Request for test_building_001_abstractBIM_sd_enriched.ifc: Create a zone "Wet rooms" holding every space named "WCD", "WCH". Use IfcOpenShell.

First a look at what the model holds.

```python
import ifcopenshell

model = ifcopenshell.open("test_building_001_abstractBIM_sd_enriched.ifc")
print(model.schema)
seen = {}
for space in model.by_type("IfcSpace"):
    seen[space.LongName] = seen.get(space.LongName, 0) + 1
for name, count in sorted(seen.items(), key=str):
    print(count, "x", name)
print("zones:", [z.Name for z in model.by_type("IfcZone")][:20])
```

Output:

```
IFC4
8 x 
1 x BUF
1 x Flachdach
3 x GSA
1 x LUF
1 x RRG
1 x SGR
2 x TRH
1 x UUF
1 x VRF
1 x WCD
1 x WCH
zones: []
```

```python
import ifcopenshell
import ifcopenshell.api.group
import ifcopenshell.api.root

model = ifcopenshell.open("test_building_001_abstractBIM_sd_enriched.ifc")

names = {"WCD", "WCH"}
spaces = [s for s in model.by_type("IfcSpace") if s.LongName in names]

zone = ifcopenshell.api.root.create_entity(model, ifc_class="IfcZone", name="Wet rooms")
ifcopenshell.api.group.assign_group(model, products=spaces, group=zone)
print(len(spaces), "spaces in", zone.Name)

model.write("test_building_001_abstractBIM_sd_enriched_v2.ifc")
```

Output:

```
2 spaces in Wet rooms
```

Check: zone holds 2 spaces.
